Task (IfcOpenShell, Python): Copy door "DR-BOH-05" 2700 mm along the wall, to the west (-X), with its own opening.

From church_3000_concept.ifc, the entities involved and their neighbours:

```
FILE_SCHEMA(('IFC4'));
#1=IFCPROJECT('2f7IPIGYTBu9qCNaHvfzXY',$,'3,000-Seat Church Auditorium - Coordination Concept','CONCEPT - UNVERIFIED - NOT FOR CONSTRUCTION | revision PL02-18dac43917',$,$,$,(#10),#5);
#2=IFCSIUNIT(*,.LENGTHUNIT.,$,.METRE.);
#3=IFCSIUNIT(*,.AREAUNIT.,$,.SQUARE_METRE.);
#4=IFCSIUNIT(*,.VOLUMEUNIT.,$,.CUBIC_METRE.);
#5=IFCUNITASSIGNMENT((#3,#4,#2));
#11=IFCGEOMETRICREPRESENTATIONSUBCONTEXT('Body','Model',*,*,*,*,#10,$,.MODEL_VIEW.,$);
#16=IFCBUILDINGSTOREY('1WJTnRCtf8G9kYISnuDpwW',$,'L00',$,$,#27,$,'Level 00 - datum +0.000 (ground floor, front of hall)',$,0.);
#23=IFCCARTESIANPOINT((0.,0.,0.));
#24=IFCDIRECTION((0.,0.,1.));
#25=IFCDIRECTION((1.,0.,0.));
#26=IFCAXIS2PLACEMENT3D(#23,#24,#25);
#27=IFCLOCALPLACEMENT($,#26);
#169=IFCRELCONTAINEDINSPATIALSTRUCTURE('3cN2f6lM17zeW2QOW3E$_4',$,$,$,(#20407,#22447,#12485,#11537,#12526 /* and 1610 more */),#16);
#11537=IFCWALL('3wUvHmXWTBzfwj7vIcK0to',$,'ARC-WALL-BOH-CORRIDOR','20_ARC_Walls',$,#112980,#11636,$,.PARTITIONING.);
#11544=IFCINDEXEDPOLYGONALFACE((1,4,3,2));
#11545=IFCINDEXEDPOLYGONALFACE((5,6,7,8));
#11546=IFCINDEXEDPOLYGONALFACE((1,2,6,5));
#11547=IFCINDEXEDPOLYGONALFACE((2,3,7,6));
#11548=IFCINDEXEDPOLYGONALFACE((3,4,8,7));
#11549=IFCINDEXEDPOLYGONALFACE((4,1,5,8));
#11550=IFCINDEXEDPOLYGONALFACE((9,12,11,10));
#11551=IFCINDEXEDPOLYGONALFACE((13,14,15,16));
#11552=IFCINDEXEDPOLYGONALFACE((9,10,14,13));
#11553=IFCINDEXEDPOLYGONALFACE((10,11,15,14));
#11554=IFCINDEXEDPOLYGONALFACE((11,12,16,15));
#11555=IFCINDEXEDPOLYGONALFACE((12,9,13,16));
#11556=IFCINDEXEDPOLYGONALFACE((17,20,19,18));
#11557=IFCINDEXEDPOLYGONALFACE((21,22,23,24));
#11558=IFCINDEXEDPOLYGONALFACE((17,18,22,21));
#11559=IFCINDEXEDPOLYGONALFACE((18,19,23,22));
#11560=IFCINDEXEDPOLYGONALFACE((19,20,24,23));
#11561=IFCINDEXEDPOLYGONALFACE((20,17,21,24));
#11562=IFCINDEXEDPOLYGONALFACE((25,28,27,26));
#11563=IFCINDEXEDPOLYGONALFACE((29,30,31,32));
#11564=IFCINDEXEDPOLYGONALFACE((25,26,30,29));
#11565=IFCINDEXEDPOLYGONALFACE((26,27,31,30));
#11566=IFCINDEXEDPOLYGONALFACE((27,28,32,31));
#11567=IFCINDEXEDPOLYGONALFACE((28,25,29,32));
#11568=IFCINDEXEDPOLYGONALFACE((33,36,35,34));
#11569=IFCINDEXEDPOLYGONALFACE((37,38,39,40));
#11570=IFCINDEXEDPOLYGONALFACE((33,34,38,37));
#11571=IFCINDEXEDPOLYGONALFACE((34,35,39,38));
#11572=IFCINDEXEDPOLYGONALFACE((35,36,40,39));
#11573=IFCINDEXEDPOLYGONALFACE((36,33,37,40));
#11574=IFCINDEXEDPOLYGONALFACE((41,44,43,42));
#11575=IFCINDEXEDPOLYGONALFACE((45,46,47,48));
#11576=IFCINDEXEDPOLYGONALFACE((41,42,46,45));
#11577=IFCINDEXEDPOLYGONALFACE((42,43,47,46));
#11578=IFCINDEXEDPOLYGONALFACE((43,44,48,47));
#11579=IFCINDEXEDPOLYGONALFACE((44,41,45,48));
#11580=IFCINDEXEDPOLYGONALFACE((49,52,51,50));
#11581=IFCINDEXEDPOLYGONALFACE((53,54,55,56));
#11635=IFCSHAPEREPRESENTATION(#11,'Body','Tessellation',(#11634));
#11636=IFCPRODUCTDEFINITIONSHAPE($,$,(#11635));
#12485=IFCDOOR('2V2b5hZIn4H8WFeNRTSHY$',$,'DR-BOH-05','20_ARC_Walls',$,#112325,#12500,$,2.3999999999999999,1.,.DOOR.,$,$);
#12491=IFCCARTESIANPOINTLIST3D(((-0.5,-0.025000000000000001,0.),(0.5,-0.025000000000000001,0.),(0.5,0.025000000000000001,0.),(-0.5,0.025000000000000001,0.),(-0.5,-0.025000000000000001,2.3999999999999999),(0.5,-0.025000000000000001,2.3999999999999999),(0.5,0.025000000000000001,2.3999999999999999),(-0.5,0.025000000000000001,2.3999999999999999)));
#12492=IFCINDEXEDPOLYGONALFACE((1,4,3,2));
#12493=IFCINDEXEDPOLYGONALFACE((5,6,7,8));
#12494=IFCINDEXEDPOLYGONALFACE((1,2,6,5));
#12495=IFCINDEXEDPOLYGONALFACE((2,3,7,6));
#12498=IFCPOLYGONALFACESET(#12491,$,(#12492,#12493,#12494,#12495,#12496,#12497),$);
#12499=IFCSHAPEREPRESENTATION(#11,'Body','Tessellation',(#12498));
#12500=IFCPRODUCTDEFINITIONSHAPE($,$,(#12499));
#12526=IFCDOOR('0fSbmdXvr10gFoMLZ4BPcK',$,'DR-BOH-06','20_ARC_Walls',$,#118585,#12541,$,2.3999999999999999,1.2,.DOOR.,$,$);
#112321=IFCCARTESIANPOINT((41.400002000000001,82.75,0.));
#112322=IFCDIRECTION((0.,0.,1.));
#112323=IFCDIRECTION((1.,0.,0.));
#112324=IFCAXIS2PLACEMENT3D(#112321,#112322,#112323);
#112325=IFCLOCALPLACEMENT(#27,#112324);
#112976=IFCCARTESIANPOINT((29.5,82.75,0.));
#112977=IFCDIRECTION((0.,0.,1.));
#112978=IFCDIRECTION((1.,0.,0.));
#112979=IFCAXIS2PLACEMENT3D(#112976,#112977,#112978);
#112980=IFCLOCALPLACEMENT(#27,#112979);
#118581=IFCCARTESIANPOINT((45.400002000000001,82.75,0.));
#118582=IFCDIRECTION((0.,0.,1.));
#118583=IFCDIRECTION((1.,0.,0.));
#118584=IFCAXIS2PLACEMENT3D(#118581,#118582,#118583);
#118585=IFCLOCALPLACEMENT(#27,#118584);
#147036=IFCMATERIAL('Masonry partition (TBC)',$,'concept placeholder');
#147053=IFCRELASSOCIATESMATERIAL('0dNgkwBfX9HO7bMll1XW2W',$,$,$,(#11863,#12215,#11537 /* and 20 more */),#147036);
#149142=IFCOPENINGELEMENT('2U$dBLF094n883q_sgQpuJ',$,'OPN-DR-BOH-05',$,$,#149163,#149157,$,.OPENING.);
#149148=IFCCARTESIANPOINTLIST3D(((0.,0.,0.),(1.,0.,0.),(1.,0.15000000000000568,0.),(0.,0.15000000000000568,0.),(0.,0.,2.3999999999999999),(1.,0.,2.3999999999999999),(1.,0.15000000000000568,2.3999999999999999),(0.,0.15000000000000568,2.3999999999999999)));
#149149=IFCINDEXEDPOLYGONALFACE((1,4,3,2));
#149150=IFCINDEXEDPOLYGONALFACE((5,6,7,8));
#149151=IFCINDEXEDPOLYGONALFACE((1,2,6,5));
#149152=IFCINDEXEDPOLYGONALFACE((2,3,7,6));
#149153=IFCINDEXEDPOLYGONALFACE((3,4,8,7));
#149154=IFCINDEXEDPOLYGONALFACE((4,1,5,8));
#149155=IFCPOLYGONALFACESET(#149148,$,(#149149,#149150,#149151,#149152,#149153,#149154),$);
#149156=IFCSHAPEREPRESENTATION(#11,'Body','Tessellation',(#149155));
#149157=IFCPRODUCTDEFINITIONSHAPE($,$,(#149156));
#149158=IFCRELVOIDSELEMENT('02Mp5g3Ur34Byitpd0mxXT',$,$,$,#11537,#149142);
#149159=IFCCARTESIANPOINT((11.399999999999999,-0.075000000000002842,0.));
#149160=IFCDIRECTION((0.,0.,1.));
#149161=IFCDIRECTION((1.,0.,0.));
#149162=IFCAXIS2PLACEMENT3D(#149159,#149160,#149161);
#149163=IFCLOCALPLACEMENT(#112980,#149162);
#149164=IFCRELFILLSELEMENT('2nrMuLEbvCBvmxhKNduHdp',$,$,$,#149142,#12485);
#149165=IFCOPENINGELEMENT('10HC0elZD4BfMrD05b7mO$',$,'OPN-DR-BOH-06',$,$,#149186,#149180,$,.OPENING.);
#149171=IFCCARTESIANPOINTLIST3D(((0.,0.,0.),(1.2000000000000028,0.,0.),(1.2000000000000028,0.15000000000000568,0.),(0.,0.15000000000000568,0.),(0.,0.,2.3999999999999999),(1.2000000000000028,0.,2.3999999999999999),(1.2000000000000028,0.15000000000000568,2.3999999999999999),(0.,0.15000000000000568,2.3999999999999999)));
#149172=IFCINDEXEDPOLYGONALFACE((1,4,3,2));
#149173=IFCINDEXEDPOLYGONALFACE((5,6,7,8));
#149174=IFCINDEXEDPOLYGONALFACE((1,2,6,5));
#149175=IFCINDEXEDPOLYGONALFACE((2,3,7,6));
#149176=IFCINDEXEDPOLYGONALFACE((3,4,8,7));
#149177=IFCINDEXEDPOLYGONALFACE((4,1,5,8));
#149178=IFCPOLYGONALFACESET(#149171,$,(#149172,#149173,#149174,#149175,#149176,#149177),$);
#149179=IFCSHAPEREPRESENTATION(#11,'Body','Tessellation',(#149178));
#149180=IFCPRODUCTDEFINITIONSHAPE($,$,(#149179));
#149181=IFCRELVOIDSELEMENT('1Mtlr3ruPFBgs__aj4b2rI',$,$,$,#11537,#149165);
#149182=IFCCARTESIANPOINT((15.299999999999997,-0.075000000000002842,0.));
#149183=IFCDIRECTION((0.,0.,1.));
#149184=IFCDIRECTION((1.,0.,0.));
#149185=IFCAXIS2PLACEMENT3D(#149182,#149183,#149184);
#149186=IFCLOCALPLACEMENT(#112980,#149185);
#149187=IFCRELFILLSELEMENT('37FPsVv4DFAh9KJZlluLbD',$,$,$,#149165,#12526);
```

```python
import ifcopenshell
import ifcopenshell.api.feature
import ifcopenshell.api.geometry
import ifcopenshell.api.root
import ifcopenshell.geom
import ifcopenshell.util.element
import ifcopenshell.util.placement
import ifcopenshell.util.shape
import ifcopenshell.util.unit

model = ifcopenshell.open("church_3000_concept.ifc")
unit_scale = ifcopenshell.util.unit.calculate_unit_scale(model)
settings = ifcopenshell.geom.settings()


def volume(element):
    """Net volume in cubic metres, openings subtracted."""
    shape = ifcopenshell.geom.create_shape(settings, element)
    return ifcopenshell.util.shape.get_volume(shape.geometry)


door = model.by_guid("2V2b5hZIn4H8WFeNRTSHY$")
opening = door.FillsVoids[0].RelatingOpeningElement
wall = opening.VoidsElements[0].RelatingBuildingElement
before = volume(wall)
shift = ifcopenshell.util.placement.get_local_placement(wall.ObjectPlacement)[:3, 0] * -2.7 / unit_scale

# copy_class copies the void relationship, type, container and properties, but no geometry.
new_opening = ifcopenshell.api.root.copy_class(model, product=opening)
new_opening.Representation = ifcopenshell.util.element.copy_deep(
    model, opening.Representation, exclude=["IfcGeometricRepresentationContext", "IfcRepresentationMap"]
)
new_door = ifcopenshell.api.root.copy_class(model, product=door)
new_door.Representation = ifcopenshell.util.element.copy_deep(
    model, door.Representation, exclude=["IfcGeometricRepresentationContext", "IfcRepresentationMap"]
)
ifcopenshell.api.feature.add_filling(model, opening=new_opening, element=new_door)

for old, new in ((opening, new_opening), (door, new_door)):
    matrix = ifcopenshell.util.placement.get_local_placement(old.ObjectPlacement)
    matrix[:3, 3] += shift
    ifcopenshell.api.geometry.edit_object_placement(model, product=new, matrix=matrix, is_si=False)

after = volume(wall)

print(f"wall volume {before:.3f} -> {after:.3f} m3")

model.write("church_3000_concept_v2.ifc")
```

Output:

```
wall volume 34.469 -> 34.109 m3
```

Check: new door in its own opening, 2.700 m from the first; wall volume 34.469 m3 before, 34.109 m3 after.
